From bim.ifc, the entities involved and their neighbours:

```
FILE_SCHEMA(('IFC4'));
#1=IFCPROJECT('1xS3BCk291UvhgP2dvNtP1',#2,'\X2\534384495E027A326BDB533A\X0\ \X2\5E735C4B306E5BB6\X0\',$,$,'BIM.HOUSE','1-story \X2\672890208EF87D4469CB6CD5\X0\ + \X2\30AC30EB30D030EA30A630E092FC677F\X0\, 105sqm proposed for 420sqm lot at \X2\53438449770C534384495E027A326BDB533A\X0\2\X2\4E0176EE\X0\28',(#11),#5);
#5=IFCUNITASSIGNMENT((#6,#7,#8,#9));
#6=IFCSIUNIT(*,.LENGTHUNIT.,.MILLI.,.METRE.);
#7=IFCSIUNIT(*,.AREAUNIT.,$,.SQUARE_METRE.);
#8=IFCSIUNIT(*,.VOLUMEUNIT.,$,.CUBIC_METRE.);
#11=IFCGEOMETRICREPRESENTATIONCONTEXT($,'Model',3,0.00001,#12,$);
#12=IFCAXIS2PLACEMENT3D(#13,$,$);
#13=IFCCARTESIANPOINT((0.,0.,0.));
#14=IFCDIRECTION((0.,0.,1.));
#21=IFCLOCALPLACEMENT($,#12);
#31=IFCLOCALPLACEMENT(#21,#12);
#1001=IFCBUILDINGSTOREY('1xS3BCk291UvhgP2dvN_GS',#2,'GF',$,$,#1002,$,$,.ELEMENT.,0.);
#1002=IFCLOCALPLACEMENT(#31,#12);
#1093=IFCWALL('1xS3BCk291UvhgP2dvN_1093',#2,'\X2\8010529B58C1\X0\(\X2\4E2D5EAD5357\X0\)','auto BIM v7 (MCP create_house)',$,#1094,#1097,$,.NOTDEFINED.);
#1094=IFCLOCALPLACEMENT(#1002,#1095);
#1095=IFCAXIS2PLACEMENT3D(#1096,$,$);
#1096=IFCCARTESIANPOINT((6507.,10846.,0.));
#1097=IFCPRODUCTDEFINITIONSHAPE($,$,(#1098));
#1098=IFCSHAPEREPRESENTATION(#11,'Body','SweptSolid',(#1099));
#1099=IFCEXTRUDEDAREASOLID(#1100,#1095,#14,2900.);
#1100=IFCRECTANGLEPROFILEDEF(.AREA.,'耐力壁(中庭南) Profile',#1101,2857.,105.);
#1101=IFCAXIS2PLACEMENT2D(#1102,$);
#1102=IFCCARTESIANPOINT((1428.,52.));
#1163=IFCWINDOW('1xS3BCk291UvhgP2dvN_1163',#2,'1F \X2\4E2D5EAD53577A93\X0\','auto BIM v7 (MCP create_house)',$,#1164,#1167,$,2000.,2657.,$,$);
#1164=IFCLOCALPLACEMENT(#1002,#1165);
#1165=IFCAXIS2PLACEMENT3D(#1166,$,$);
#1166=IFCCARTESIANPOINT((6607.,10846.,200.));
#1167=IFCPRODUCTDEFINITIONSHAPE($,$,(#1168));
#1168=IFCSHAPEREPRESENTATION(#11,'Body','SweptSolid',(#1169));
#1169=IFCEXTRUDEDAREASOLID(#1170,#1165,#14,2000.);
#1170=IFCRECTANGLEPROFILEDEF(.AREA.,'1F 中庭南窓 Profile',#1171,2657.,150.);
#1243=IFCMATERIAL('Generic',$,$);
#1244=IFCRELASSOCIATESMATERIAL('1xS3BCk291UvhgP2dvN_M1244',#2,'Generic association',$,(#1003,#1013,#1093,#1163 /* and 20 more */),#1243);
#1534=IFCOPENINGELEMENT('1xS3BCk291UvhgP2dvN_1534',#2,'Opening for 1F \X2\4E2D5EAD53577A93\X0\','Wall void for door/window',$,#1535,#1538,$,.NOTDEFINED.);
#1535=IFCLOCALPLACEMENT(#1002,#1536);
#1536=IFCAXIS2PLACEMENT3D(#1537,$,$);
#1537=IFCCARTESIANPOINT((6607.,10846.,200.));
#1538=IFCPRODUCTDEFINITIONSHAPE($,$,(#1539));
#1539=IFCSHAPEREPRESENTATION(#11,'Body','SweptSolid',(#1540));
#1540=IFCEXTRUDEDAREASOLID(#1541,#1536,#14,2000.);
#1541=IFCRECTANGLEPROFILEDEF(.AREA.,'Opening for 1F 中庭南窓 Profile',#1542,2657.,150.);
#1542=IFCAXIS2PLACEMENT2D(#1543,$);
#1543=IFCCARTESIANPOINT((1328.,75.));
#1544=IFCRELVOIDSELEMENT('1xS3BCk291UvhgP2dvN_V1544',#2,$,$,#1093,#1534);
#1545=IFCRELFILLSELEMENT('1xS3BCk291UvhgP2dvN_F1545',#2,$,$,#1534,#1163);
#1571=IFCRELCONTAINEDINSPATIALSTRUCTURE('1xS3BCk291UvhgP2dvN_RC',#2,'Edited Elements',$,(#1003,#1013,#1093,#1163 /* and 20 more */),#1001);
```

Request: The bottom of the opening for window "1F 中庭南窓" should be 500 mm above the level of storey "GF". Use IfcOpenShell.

```python
import numpy as np
import ifcopenshell
import ifcopenshell.api.geometry
import ifcopenshell.geom
import ifcopenshell.util.element
import ifcopenshell.util.placement
import ifcopenshell.util.shape
import ifcopenshell.util.unit

model = ifcopenshell.open("bim.ifc")
unit_scale = ifcopenshell.util.unit.calculate_unit_scale(model)

window = model.by_id(1163)
opening = window.FillsVoids[0].RelatingOpeningElement
storey = ifcopenshell.util.element.get_container(window, ifc_class="IfcBuildingStorey")
level = ifcopenshell.util.placement.get_local_placement(storey.ObjectPlacement)[2, 3]

# The opening's origin need not be at the sill, so measure its lowest point.
shape = ifcopenshell.geom.create_shape(ifcopenshell.geom.settings(), opening)
bottom = ifcopenshell.util.shape.get_shape_bottom_elevation(shape, shape.geometry) / unit_scale
dz = level + 500.0 - bottom

shift = np.array([0.0, 0.0, dz])
# The window is not placed relative to its opening, so move both.
for product in (opening, window):
    matrix = ifcopenshell.util.placement.get_local_placement(product.ObjectPlacement)
    matrix[:3, 3] += shift
    ifcopenshell.api.geometry.edit_object_placement(model, product=product, matrix=matrix, is_si=False)

print(f"moved by {dz * unit_scale:+.3f} m")

model.write("bim_edited.ifc")
```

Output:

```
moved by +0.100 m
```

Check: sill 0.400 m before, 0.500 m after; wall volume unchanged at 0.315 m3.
